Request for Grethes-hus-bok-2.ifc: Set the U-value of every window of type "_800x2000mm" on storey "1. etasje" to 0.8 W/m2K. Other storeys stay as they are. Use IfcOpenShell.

First a look at what the model holds.

```python
import ifcopenshell
import ifcopenshell.util.element

model = ifcopenshell.open("Grethes-hus-bok-2.ifc")
print(model.schema)
storey = next(s for s in model.by_type("IfcBuildingStorey") if s.Name == "1. etasje")
windows = [e for e in ifcopenshell.util.element.get_decomposition(storey) if e.is_a("IfcWindow")]
seen = {}
for e in windows:
    element_type = ifcopenshell.util.element.get_type(e)
    key = (element_type.Name if element_type != e and element_type else None, ifcopenshell.util.element.get_pset(e, "Pset_WindowCommon", "ThermalTransmittance"))
    seen[key] = seen.get(key, 0) + 1
for (name, value), count in sorted(seen.items(), key=str):
    print(count, "x", name, "|", value)
```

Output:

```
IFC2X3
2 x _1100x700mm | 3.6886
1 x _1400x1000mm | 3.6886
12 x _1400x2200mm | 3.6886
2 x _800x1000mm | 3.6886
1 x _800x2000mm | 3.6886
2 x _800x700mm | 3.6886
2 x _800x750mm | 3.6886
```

```python
import ifcopenshell
import ifcopenshell.api.pset
import ifcopenshell.util.element

model = ifcopenshell.open("Grethes-hus-bok-2.ifc")

storey = next(s for s in model.by_type("IfcBuildingStorey") if s.Name == "1. etasje")
windows = [e for e in ifcopenshell.util.element.get_decomposition(storey) if e.is_a("IfcWindow")]

count = 0
for e in windows:
    element_type = ifcopenshell.util.element.get_type(e)
    if element_type in (None, e) or element_type.Name != "_800x2000mm":
        continue
    # add_pset returns the element's existing set when there is one.
    pset = ifcopenshell.api.pset.add_pset(model, product=e, name="Pset_WindowCommon")
    ifcopenshell.api.pset.edit_pset(model, pset=pset, properties={"ThermalTransmittance": 0.8})
    count += 1

print(count, "windows updated")

model.write("Grethes-hus-bok-2-out.ifc")
```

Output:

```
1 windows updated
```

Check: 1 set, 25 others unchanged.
